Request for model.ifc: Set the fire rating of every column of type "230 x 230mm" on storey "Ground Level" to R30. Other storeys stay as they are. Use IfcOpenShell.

First a look at what the model holds.

```python
import ifcopenshell
import ifcopenshell.util.element

model = ifcopenshell.open("model.ifc")
print(model.schema)
storey = next(s for s in model.by_type("IfcBuildingStorey") if s.Name == "Ground Level")
columns = [e for e in ifcopenshell.util.element.get_decomposition(storey) if e.is_a("IfcColumn")]
seen = {}
for e in columns:
    element_type = ifcopenshell.util.element.get_type(e)
    key = (element_type.Name if element_type != e and element_type else None, ifcopenshell.util.element.get_pset(e, "Pset_ColumnCommon", "FireRating"))
    seen[key] = seen.get(key, 0) + 1
for (name, value), count in sorted(seen.items(), key=str):
    print(count, "x", name, "|", value)
```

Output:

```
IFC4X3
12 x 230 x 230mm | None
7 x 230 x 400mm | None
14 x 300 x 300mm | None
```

```python
import ifcopenshell
import ifcopenshell.api.pset
import ifcopenshell.util.element

model = ifcopenshell.open("model.ifc")

storey = next(s for s in model.by_type("IfcBuildingStorey") if s.Name == "Ground Level")
columns = [e for e in ifcopenshell.util.element.get_decomposition(storey) if e.is_a("IfcColumn")]

count = 0
for e in columns:
    element_type = ifcopenshell.util.element.get_type(e)
    if element_type in (None, e) or element_type.Name != "230 x 230mm":
        continue
    # add_pset returns the element's existing set when there is one.
    pset = ifcopenshell.api.pset.add_pset(model, product=e, name="Pset_ColumnCommon")
    ifcopenshell.api.pset.edit_pset(model, pset=pset, properties={"FireRating": "R30"})
    count += 1

print(count, "columns updated")

model.write("model_edited.ifc")
```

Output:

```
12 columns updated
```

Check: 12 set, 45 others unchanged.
